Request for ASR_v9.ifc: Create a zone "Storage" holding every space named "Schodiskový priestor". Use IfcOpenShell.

First a look at what the model holds.

```python
import ifcopenshell

model = ifcopenshell.open("ASR_v9.ifc")
print(model.schema)
seen = {}
for space in model.by_type("IfcSpace"):
    seen[space.LongName] = seen.get(space.LongName, 0) + 1
for name, count in sorted(seen.items(), key=str):
    print(count, "x", name)
print("zones:", [z.Name for z in model.by_type("IfcZone")][:20])
```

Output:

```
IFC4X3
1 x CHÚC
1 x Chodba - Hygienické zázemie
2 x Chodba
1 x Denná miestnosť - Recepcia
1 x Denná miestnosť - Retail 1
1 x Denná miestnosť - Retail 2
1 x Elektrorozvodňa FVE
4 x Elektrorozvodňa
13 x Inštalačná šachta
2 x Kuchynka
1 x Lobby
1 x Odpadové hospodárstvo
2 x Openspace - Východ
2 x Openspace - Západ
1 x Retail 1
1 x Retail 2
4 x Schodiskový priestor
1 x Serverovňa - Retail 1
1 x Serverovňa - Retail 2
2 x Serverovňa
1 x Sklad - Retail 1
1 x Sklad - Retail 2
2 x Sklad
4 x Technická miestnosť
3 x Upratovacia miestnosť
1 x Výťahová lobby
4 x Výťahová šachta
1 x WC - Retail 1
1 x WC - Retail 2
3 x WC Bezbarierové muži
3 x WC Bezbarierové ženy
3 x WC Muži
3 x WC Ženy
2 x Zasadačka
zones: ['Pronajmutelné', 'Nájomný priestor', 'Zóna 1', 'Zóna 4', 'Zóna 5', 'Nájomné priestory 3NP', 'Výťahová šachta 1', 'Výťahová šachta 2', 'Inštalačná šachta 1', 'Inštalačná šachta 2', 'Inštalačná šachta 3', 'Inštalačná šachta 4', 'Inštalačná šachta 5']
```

```python
import ifcopenshell
import ifcopenshell.api.group
import ifcopenshell.api.root

model = ifcopenshell.open("ASR_v9.ifc")

names = {"Schodiskový priestor"}
spaces = [s for s in model.by_type("IfcSpace") if s.LongName in names]

zone = ifcopenshell.api.root.create_entity(model, ifc_class="IfcZone", name="Storage")
ifcopenshell.api.group.assign_group(model, products=spaces, group=zone)
print(len(spaces), "spaces in", zone.Name)

model.write("ASR_v9-out.ifc")
```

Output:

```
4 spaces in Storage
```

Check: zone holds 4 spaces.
